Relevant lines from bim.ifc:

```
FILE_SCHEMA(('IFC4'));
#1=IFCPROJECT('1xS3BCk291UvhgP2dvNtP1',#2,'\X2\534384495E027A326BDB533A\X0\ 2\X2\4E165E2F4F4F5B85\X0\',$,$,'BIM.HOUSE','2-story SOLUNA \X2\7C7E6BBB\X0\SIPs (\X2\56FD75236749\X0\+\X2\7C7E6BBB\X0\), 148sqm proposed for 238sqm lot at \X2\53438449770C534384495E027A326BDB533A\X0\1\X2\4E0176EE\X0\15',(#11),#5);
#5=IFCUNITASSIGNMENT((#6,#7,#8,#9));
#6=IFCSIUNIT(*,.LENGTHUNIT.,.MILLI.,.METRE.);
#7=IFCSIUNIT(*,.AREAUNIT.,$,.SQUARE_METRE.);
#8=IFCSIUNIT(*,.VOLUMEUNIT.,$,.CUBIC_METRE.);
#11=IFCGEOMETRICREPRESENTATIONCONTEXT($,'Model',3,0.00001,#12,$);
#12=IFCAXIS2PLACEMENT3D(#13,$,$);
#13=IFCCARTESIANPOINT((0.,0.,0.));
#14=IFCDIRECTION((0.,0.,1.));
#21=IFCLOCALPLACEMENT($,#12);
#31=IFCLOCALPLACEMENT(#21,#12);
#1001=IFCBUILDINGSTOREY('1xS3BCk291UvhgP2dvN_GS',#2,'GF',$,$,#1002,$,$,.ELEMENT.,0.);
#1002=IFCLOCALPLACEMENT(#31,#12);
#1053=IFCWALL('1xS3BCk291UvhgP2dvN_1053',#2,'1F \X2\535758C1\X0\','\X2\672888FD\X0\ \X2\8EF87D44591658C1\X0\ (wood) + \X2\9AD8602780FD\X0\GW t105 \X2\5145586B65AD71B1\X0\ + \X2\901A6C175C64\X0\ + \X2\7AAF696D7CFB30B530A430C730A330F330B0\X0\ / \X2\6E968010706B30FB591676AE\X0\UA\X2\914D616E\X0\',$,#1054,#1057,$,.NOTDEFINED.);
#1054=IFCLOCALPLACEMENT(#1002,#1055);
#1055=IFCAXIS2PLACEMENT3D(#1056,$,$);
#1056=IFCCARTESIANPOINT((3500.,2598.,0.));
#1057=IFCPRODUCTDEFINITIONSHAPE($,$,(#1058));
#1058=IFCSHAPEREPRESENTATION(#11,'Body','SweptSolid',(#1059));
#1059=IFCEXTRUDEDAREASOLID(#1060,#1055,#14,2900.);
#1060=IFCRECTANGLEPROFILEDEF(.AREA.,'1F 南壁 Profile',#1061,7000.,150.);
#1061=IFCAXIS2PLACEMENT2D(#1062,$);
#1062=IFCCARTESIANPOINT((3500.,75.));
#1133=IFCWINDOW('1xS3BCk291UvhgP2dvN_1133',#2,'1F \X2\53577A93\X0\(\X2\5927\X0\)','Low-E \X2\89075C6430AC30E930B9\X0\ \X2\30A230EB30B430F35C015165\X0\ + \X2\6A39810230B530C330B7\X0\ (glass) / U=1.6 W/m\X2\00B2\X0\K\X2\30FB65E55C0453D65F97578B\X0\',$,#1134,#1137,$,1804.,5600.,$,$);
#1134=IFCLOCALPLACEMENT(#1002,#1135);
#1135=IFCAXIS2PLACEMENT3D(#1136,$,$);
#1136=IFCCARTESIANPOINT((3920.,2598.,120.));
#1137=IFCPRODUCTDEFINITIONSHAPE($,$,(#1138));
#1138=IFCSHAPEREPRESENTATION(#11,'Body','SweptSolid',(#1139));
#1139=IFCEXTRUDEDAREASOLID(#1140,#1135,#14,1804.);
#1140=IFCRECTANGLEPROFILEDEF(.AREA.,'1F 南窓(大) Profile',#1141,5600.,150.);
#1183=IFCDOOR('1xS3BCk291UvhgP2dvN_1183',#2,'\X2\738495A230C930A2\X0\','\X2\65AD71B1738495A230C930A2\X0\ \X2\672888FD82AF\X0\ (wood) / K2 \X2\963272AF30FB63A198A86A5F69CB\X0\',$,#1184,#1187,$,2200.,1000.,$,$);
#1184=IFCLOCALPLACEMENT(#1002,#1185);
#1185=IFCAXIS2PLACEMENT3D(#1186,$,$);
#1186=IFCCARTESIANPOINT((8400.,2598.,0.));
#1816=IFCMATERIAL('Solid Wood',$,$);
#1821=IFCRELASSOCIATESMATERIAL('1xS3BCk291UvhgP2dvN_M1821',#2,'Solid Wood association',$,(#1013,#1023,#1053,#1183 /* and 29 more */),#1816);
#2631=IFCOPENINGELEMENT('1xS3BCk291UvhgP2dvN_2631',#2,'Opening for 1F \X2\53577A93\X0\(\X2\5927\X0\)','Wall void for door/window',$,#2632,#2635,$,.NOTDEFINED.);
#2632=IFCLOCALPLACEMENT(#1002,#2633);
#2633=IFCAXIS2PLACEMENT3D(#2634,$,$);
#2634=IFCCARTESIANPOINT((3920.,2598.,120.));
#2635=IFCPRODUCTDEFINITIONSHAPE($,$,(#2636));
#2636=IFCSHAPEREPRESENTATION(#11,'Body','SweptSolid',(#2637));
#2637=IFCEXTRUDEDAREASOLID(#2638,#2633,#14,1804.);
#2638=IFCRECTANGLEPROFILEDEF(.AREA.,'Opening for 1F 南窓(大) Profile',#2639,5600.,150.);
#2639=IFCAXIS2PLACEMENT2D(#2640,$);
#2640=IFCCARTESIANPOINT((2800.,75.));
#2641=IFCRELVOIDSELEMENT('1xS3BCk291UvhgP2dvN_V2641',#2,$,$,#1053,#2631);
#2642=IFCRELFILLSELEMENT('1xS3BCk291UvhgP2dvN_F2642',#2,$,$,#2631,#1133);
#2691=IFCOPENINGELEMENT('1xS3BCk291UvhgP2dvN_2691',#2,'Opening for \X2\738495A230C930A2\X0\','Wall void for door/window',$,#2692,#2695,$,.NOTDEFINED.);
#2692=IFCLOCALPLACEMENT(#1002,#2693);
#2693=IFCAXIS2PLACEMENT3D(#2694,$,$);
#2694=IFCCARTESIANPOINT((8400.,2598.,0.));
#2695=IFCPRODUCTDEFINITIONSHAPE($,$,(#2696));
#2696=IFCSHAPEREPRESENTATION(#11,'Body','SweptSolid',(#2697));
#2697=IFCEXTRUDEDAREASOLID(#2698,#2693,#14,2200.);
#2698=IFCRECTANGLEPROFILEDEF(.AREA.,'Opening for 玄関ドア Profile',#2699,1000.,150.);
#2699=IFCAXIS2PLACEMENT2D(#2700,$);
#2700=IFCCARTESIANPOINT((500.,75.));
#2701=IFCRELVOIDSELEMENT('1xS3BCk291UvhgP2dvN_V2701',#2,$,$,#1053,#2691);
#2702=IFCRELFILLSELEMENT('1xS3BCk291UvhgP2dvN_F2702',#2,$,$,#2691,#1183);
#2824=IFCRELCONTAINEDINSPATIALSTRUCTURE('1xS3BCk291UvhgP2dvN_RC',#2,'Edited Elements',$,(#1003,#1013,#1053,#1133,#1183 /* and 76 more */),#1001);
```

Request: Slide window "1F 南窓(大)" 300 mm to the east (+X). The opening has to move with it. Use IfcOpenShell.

```python
import ifcopenshell
import ifcopenshell.api.geometry
import ifcopenshell.util.placement

model = ifcopenshell.open("bim.ifc")

window = model.by_id(1133)
opening = window.FillsVoids[0].RelatingOpeningElement
wall = opening.VoidsElements[0].RelatingBuildingElement

wall_matrix = ifcopenshell.util.placement.get_local_placement(wall.ObjectPlacement)
shift = wall_matrix[:3, 0] * 300.0
before = ifcopenshell.util.placement.get_local_placement(window.ObjectPlacement)[:3, 3].copy()

# The window is not placed relative to its opening, so move both.
for product in (opening, window):
    matrix = ifcopenshell.util.placement.get_local_placement(product.ObjectPlacement)
    matrix[:3, 3] += shift
    ifcopenshell.api.geometry.edit_object_placement(model, product=product, matrix=matrix, is_si=False)

after = ifcopenshell.util.placement.get_local_placement(window.ObjectPlacement)[:3, 3]
print("window moved by", (after - before).round(3) + 0.0)

model.write("bim_updated.ifc")
```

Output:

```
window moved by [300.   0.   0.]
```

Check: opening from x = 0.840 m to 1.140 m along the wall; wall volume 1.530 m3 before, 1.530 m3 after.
